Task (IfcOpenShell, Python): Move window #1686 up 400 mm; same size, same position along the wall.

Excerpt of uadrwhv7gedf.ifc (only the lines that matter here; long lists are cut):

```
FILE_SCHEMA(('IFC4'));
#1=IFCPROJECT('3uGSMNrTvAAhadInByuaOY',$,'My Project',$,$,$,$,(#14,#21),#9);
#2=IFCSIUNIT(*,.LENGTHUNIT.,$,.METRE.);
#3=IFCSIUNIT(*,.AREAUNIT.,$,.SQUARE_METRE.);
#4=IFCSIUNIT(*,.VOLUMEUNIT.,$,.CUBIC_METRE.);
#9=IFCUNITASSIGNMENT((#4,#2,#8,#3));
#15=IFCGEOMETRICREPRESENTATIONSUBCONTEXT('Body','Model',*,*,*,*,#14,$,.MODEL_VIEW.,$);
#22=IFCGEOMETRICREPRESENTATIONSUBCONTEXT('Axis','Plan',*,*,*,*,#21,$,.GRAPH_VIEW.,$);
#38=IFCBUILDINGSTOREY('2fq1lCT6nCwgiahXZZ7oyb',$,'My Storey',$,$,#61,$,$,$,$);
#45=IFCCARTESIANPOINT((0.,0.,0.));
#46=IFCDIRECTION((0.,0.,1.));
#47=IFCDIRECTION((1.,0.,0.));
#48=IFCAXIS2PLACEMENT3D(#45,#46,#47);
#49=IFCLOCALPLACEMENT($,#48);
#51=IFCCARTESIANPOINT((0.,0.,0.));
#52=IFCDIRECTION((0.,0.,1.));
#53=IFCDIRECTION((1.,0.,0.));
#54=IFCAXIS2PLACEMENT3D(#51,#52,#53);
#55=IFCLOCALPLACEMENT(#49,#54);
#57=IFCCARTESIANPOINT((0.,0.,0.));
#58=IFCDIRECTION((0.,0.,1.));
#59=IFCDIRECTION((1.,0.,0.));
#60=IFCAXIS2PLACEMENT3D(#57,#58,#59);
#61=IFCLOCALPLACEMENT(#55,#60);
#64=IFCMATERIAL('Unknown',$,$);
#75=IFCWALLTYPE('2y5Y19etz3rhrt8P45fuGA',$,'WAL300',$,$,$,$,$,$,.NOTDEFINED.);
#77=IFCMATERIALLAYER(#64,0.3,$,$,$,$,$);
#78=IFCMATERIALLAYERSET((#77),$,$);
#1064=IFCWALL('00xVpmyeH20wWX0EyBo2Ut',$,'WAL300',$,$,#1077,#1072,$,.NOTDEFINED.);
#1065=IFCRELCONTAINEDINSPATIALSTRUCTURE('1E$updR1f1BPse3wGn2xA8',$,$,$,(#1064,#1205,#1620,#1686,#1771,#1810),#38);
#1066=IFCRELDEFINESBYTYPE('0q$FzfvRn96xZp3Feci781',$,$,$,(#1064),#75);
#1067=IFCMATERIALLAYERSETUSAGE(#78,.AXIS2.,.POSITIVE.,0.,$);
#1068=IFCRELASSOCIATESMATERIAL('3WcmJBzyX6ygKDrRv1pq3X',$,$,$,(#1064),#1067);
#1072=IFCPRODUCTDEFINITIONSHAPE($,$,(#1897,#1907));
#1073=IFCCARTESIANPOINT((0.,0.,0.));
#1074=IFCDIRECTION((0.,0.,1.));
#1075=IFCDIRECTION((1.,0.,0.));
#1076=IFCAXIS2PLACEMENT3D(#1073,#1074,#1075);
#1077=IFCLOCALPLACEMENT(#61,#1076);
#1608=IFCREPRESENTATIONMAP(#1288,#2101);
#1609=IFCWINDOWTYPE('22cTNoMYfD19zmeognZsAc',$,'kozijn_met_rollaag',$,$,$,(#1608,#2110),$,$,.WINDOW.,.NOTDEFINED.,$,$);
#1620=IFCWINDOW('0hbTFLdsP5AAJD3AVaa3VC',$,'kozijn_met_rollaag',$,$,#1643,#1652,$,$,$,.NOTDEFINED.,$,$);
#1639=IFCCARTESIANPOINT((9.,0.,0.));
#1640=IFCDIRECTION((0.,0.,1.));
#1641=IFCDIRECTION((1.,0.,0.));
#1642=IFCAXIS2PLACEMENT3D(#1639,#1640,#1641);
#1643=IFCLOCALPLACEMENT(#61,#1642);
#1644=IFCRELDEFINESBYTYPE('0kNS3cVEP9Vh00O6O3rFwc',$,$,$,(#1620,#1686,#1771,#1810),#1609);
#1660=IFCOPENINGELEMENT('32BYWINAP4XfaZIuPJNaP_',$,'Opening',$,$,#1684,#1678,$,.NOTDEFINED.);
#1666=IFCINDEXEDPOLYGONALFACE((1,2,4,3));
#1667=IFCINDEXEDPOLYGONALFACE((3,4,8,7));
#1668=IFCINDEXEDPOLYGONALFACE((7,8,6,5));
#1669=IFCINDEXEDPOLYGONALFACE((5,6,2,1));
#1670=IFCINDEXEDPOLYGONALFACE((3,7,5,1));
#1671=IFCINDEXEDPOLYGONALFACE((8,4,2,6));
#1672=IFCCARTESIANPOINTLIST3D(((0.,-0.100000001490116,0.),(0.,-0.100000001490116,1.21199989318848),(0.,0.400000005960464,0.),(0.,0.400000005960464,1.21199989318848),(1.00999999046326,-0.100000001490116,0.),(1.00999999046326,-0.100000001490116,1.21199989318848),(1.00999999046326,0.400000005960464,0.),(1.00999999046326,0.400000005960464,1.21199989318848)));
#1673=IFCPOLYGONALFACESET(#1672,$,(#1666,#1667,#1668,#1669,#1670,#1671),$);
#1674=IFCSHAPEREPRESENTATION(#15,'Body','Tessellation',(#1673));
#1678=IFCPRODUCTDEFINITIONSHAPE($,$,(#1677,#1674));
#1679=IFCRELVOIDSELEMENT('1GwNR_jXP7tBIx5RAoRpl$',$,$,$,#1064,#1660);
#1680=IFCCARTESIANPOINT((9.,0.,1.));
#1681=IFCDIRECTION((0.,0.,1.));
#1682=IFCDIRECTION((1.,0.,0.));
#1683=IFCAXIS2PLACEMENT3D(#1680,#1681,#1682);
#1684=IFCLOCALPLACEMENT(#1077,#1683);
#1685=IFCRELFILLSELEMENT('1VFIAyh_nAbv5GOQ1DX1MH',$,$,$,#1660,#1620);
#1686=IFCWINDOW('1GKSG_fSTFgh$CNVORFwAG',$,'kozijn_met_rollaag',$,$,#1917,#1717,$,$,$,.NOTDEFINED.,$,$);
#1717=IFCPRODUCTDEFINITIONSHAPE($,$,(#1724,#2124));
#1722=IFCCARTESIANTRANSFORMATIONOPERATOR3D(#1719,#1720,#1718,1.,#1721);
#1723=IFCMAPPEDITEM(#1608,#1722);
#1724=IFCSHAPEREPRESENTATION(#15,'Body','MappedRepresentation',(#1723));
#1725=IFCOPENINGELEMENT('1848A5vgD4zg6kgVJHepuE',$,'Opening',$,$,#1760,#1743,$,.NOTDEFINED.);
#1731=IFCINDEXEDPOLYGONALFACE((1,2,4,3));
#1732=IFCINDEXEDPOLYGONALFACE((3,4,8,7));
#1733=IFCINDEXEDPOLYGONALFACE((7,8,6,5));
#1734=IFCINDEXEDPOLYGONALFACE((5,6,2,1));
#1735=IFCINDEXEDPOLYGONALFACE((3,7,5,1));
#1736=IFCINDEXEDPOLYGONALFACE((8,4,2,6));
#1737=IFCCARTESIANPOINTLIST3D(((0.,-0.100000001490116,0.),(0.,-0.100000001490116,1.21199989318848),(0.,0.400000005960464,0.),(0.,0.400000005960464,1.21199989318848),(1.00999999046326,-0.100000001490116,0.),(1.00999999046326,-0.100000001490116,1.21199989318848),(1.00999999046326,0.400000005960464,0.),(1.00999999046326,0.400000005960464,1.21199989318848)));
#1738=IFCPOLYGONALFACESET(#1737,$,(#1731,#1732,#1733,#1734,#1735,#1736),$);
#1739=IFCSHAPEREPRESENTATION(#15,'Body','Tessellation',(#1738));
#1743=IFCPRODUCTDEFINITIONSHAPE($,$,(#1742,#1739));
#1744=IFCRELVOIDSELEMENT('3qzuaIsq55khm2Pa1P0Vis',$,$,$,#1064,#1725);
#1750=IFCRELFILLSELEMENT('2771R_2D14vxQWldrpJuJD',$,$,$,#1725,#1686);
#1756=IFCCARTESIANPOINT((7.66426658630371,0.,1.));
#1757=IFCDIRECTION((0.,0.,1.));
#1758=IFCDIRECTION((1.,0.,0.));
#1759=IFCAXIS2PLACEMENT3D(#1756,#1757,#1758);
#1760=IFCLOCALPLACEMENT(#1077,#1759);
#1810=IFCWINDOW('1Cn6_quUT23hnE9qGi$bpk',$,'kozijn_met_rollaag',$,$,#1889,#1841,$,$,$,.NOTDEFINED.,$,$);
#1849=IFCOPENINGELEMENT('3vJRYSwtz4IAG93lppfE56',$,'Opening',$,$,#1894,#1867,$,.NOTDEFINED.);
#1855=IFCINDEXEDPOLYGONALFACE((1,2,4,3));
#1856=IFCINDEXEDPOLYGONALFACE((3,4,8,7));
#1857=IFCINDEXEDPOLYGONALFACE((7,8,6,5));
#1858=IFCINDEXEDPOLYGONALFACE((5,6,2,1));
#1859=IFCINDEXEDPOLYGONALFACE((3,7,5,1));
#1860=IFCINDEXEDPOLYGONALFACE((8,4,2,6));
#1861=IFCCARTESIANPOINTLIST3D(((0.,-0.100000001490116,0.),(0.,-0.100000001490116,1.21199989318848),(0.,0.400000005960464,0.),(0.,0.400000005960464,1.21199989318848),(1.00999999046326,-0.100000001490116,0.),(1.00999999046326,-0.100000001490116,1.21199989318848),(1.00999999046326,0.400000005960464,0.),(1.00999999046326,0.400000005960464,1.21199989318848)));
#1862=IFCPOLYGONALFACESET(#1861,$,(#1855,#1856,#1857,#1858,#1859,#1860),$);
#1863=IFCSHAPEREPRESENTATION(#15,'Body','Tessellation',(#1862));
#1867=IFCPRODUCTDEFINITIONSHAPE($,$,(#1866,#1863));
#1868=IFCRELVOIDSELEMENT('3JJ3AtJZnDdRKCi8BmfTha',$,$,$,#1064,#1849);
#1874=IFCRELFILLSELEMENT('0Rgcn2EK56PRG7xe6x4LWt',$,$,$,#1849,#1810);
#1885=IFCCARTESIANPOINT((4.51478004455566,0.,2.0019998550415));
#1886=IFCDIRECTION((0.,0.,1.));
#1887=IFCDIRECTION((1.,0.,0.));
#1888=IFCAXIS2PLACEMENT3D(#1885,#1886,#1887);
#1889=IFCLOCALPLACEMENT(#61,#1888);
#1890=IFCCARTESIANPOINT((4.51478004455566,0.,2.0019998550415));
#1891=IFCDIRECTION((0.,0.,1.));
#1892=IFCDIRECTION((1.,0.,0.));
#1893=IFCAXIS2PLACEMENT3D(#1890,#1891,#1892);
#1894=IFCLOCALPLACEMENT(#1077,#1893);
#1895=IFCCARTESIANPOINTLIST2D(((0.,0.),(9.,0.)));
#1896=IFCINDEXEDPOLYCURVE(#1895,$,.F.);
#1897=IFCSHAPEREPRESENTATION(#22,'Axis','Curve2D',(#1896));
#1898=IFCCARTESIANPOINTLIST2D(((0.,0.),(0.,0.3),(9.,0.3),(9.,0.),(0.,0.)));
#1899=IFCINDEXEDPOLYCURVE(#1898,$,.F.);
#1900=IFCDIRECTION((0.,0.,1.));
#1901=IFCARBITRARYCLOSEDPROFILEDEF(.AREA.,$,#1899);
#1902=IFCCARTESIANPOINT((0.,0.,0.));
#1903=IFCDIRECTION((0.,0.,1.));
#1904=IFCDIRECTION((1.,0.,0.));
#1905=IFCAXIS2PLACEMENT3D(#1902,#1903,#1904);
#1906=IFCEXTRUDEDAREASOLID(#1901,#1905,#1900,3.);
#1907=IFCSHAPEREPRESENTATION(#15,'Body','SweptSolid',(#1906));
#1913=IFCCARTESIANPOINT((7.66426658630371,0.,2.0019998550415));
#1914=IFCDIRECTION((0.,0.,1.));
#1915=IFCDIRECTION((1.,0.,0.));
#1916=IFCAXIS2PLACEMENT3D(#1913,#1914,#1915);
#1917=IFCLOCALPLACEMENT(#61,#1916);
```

```python
import numpy as np
import ifcopenshell
import ifcopenshell.api.geometry
import ifcopenshell.util.placement
import ifcopenshell.util.unit

model = ifcopenshell.open("uadrwhv7gedf.ifc")
unit_scale = ifcopenshell.util.unit.calculate_unit_scale(model)

window = model.by_guid("1GKSG_fSTFgh$CNVORFwAG")
opening = window.FillsVoids[0].RelatingOpeningElement
dz = 0.4 / unit_scale

shift = np.array([0.0, 0.0, dz])
# The window is not placed relative to its opening, so move both.
for product in (opening, window):
    matrix = ifcopenshell.util.placement.get_local_placement(product.ObjectPlacement)
    matrix[:3, 3] += shift
    ifcopenshell.api.geometry.edit_object_placement(model, product=product, matrix=matrix, is_si=False)

print(f"moved by {dz * unit_scale:+.3f} m")

model.write("uadrwhv7gedf_updated.ifc")
```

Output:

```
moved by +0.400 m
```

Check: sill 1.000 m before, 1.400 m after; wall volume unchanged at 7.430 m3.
